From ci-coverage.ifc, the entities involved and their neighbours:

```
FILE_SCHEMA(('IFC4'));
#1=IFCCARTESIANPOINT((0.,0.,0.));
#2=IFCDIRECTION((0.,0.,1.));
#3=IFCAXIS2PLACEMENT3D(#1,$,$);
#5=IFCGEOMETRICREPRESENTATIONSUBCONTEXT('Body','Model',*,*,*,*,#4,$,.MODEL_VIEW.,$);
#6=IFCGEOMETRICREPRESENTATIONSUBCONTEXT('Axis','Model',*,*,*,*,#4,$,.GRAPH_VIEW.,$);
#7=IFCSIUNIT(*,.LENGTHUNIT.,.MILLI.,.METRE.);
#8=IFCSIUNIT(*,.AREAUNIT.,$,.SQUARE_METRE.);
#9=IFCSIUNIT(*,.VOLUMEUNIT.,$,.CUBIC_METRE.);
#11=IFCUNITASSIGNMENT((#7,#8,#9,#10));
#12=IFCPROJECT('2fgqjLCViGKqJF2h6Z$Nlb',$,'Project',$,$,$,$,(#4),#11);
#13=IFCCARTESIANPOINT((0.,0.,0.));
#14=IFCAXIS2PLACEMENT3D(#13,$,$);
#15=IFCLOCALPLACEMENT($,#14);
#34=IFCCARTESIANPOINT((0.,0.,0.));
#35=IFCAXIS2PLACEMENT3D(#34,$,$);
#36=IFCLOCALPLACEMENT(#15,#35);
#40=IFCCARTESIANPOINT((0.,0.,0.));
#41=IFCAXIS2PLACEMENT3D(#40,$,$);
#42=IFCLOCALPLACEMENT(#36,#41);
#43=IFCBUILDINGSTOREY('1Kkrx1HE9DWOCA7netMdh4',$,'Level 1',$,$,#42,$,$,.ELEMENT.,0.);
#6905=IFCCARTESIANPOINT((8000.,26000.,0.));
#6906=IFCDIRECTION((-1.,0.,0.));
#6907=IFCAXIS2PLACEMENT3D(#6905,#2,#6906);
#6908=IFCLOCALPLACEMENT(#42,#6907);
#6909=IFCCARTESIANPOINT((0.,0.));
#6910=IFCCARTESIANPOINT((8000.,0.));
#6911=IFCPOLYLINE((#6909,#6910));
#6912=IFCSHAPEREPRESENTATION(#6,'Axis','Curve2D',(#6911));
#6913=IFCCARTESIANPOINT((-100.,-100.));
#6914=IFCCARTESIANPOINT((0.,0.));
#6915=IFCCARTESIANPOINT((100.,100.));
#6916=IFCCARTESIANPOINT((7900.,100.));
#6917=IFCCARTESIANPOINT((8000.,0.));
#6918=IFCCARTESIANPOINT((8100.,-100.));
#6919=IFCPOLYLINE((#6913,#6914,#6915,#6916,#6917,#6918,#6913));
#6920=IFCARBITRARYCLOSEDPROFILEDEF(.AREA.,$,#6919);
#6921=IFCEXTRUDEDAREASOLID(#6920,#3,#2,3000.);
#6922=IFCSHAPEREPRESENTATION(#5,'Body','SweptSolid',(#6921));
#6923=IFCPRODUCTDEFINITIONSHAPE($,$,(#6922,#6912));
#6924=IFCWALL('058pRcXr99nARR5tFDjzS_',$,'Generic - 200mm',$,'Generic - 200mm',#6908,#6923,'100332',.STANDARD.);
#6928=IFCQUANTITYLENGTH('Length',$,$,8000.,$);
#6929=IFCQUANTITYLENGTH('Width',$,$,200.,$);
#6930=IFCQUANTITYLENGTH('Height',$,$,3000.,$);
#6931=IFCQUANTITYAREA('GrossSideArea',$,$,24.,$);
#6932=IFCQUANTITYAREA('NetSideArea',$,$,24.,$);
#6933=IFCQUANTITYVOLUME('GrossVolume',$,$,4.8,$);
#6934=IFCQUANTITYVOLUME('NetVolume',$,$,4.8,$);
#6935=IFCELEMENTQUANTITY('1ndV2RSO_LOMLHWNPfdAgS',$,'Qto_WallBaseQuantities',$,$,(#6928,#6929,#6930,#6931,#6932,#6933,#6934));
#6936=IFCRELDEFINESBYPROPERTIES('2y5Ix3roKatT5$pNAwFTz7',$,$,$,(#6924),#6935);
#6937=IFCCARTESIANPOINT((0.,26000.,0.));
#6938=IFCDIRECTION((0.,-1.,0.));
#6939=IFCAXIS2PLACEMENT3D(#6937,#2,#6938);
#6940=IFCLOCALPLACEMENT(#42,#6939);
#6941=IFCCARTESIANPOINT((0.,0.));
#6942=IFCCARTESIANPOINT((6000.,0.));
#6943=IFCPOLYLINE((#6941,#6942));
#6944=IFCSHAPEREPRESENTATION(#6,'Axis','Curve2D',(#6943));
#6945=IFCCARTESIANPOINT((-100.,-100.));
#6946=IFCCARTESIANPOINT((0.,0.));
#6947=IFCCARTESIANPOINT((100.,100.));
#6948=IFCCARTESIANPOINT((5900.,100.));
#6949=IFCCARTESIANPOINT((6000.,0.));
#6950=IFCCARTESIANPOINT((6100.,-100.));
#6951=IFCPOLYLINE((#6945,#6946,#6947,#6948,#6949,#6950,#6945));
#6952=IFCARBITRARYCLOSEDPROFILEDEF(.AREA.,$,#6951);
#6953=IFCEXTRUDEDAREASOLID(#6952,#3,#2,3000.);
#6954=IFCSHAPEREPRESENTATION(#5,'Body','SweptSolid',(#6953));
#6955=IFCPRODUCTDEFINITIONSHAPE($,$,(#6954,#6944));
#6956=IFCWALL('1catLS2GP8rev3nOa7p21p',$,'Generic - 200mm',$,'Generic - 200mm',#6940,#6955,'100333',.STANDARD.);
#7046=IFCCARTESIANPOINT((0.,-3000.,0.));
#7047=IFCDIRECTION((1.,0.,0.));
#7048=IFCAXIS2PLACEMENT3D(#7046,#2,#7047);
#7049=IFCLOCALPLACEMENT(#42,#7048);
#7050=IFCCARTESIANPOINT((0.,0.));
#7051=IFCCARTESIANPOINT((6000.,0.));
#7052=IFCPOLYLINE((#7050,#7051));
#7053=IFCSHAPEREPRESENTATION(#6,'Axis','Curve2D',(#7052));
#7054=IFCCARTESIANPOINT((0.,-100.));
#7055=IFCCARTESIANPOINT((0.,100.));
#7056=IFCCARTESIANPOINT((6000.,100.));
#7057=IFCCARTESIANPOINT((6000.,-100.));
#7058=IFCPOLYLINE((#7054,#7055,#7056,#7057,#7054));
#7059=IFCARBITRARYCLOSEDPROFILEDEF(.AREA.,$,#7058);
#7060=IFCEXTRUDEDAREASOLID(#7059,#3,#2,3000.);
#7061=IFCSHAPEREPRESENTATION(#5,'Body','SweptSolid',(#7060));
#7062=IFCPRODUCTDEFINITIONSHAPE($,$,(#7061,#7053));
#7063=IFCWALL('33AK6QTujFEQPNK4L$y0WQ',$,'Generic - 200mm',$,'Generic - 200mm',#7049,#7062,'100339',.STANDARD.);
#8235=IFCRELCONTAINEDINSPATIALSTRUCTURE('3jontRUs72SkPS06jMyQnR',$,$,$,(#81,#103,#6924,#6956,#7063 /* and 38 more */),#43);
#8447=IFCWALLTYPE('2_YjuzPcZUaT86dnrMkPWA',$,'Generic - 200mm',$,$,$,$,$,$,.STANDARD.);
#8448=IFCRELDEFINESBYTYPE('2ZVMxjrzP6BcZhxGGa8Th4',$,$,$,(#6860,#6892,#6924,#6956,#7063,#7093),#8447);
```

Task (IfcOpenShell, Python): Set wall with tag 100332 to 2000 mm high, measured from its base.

```python
import ifcopenshell
import ifcopenshell.api.pset
import ifcopenshell.geom
import ifcopenshell.util.element
import ifcopenshell.util.representation
import ifcopenshell.util.shape
import ifcopenshell.util.unit

model = ifcopenshell.open("ci-coverage.ifc")
unit_scale = ifcopenshell.util.unit.calculate_unit_scale(model)
area_scale = ifcopenshell.util.unit.calculate_unit_scale(model, "AREAUNIT")
volume_scale = ifcopenshell.util.unit.calculate_unit_scale(model, "VOLUMEUNIT")
settings = ifcopenshell.geom.settings()


def volume(element):
    """Net volume in cubic metres, openings subtracted."""
    shape = ifcopenshell.geom.create_shape(settings, element)
    return ifcopenshell.util.shape.get_volume(shape.geometry)


wall = model.by_guid("058pRcXr99nARR5tFDjzS_")
before = volume(wall)

body = ifcopenshell.util.representation.get_representation(wall, "Model", "Body")
solid = body.Items[0]
old_height = solid.Depth
solid.Depth = 2000.0
after = volume(wall)
thickness = 0.2  # wall thickness in metres

# Update the stored height, areas and volumes.
qto = model.by_id(ifcopenshell.util.element.get_pset(wall, "Qto_WallBaseQuantities", should_inherit=False)["id"])
ifcopenshell.api.pset.edit_qto(model, qto=qto, properties={
    "Height": solid.Depth,
    "GrossSideArea": ifcopenshell.util.element.get_pset(wall, "Qto_WallBaseQuantities", "GrossSideArea") * solid.Depth / old_height,
    "NetSideArea": after / thickness / area_scale,
    "GrossVolume": ifcopenshell.util.element.get_pset(wall, "Qto_WallBaseQuantities", "GrossVolume") * solid.Depth / old_height,
    "NetVolume": after / volume_scale,
})

print(f"height {old_height:g} -> {solid.Depth:g}, volume {before:.3f} -> {after:.3f} m3")

model.write("ci-coverage-out.ifc")
```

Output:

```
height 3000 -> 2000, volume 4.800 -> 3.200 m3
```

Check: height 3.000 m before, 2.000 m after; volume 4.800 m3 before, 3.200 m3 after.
